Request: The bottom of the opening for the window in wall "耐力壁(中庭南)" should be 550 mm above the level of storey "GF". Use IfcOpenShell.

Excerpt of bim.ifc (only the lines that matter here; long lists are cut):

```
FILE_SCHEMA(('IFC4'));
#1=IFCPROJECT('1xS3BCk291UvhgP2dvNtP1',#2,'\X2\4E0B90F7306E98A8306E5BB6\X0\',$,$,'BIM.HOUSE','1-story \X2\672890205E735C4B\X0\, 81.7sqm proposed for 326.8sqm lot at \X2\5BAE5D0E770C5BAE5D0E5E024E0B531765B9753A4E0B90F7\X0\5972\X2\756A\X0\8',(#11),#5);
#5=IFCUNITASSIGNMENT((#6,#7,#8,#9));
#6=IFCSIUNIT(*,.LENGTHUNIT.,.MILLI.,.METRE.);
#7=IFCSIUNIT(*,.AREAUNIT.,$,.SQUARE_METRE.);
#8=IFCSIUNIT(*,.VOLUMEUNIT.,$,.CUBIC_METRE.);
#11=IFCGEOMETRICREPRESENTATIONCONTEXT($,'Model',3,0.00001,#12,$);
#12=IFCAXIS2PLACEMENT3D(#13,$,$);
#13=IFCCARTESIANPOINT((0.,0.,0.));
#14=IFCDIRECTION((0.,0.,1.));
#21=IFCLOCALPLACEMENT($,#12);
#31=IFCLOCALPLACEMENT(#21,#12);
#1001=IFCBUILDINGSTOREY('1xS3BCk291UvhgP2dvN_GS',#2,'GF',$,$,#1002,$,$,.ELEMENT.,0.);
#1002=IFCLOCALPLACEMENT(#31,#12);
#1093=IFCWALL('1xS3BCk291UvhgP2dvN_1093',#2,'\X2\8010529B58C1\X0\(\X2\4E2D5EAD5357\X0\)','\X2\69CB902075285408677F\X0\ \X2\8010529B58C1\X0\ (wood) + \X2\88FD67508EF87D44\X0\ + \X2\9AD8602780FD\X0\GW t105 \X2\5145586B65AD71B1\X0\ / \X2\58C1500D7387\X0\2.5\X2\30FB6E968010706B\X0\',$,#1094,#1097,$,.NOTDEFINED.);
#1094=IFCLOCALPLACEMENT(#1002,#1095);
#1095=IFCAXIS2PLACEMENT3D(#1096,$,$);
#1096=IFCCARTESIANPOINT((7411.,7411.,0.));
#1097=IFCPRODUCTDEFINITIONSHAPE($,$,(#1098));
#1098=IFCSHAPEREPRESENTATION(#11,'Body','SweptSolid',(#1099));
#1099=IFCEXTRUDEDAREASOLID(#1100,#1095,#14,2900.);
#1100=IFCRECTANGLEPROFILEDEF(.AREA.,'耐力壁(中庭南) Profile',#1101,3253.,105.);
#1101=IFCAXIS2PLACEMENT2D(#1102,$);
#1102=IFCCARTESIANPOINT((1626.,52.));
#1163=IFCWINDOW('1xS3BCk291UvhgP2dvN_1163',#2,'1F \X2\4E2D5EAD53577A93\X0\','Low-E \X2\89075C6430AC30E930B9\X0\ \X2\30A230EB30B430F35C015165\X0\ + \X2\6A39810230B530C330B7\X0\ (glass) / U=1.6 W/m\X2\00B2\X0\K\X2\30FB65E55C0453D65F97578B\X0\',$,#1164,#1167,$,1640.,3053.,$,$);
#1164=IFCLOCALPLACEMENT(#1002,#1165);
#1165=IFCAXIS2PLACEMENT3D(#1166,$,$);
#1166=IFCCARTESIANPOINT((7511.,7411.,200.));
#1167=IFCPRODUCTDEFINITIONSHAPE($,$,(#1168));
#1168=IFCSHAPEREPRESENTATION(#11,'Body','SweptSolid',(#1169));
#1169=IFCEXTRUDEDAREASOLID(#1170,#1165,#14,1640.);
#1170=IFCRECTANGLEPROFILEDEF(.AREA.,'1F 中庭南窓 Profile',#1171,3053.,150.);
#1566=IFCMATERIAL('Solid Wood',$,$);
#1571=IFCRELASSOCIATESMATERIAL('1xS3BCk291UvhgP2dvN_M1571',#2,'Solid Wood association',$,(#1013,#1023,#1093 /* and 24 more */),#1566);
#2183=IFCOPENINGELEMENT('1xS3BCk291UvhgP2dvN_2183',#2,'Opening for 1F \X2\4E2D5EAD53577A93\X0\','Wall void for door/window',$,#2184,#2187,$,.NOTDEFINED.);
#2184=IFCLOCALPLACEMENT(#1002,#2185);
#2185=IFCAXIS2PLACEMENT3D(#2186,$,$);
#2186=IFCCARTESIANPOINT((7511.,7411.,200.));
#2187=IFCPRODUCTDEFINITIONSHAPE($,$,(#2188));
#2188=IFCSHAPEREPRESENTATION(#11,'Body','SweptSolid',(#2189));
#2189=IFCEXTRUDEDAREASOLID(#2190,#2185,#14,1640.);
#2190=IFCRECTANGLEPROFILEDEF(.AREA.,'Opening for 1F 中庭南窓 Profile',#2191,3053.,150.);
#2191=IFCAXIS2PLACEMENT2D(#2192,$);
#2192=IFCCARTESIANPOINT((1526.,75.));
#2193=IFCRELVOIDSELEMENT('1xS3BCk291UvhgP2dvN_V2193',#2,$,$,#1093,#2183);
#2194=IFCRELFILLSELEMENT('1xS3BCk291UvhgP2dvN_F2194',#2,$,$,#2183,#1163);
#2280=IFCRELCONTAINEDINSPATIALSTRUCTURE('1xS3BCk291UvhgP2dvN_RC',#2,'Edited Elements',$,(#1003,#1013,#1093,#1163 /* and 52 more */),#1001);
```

```python
import numpy as np
import ifcopenshell
import ifcopenshell.api.geometry
import ifcopenshell.geom
import ifcopenshell.util.element
import ifcopenshell.util.placement
import ifcopenshell.util.shape
import ifcopenshell.util.unit

model = ifcopenshell.open("bim.ifc")
unit_scale = ifcopenshell.util.unit.calculate_unit_scale(model)

window = model.by_guid("1xS3BCk291UvhgP2dvN_1163")
opening = window.FillsVoids[0].RelatingOpeningElement
storey = ifcopenshell.util.element.get_container(window, ifc_class="IfcBuildingStorey")
level = ifcopenshell.util.placement.get_local_placement(storey.ObjectPlacement)[2, 3]

# The opening's origin need not be at the sill, so measure its lowest point.
shape = ifcopenshell.geom.create_shape(ifcopenshell.geom.settings(), opening)
bottom = ifcopenshell.util.shape.get_shape_bottom_elevation(shape, shape.geometry) / unit_scale
dz = level + 550.0 - bottom

shift = np.array([0.0, 0.0, dz])
# The window is not placed relative to its opening, so move both.
for product in (opening, window):
    matrix = ifcopenshell.util.placement.get_local_placement(product.ObjectPlacement)
    matrix[:3, 3] += shift
    ifcopenshell.api.geometry.edit_object_placement(model, product=product, matrix=matrix, is_si=False)

print(f"moved by {dz * unit_scale:+.3f} m")

model.write("bim_rev.ifc")
```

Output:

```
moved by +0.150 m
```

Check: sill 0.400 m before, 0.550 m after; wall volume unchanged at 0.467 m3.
